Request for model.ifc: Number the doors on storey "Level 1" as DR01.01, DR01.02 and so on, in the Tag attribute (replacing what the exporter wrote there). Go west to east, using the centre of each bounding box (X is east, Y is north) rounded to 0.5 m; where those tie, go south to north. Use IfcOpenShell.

First a look at what the model holds.

```python
import ifcopenshell
import ifcopenshell.util.element
import ifcopenshell.util.placement

model = ifcopenshell.open("model.ifc")
print(model.schema)
storey = next(s for s in model.by_type("IfcBuildingStorey") if s.Name == "Level 1")
doors = [e for e in ifcopenshell.util.element.get_decomposition(storey) if e.is_a("IfcDoor")]
for e in sorted(doors, key=lambda e: e.id()):
    origin = ifcopenshell.util.placement.get_local_placement(e.ObjectPlacement)[:3, 3]
    print(e.id(), e.Tag, e.Name, origin.round(2) + 0.0, sep=" | ")
```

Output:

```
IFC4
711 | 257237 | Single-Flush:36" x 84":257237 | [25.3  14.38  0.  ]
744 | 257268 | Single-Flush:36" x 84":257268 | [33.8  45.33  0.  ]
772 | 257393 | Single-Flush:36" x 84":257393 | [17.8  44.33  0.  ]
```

```python
import ifcopenshell
import ifcopenshell.geom
import ifcopenshell.util.element
import ifcopenshell.util.shape

model = ifcopenshell.open("model.ifc")
settings = ifcopenshell.geom.settings()
settings.set("use-world-coords", True)


def centre(element):
    shape = ifcopenshell.geom.create_shape(settings, element)
    return ifcopenshell.util.shape.get_bbox_centroid(shape.geometry)


storey = next(s for s in model.by_type("IfcBuildingStorey") if s.Name == "Level 1")
doors = [e for e in ifcopenshell.util.element.get_decomposition(storey) if e.is_a("IfcDoor")]

# Insertion points can sit at a corner or the storey origin, so sort by the geometry (in metres).
centres = {e: centre(e) for e in doors}
doors.sort(key=lambda e: (round(centres[e][0] / 0.5), centres[e][1]))

for i, e in enumerate(doors, start=1):
    number = f"DR01.{i:02d}"
    e.Tag = number
    print(e.id(), number)

model.write("model_v2.ifc")
```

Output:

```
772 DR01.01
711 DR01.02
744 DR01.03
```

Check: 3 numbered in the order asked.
